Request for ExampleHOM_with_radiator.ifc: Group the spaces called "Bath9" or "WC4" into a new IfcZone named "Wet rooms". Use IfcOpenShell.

First a look at what the model holds.

```python
import ifcopenshell

model = ifcopenshell.open("ExampleHOM_with_radiator.ifc")
print(model.schema)
seen = {}
for space in model.by_type("IfcSpace"):
    seen[space.Name] = seen.get(space.Name, 0) + 1
for name, count in sorted(seen.items(), key=str):
    print(count, "x", name)
print("zones:", [z.Name for z in model.by_type("IfcZone")][:20])
```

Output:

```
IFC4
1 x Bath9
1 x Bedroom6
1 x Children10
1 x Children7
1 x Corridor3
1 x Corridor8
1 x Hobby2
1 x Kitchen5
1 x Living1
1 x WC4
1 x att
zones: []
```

```python
import ifcopenshell
import ifcopenshell.api.group
import ifcopenshell.api.root

model = ifcopenshell.open("ExampleHOM_with_radiator.ifc")

names = {"Bath9", "WC4"}
spaces = [s for s in model.by_type("IfcSpace") if s.Name in names]

zone = ifcopenshell.api.root.create_entity(model, ifc_class="IfcZone", name="Wet rooms")
ifcopenshell.api.group.assign_group(model, products=spaces, group=zone)
print(len(spaces), "spaces in", zone.Name)

model.write("ExampleHOM_with_radiator_v2.ifc")
```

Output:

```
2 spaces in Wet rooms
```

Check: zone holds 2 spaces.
